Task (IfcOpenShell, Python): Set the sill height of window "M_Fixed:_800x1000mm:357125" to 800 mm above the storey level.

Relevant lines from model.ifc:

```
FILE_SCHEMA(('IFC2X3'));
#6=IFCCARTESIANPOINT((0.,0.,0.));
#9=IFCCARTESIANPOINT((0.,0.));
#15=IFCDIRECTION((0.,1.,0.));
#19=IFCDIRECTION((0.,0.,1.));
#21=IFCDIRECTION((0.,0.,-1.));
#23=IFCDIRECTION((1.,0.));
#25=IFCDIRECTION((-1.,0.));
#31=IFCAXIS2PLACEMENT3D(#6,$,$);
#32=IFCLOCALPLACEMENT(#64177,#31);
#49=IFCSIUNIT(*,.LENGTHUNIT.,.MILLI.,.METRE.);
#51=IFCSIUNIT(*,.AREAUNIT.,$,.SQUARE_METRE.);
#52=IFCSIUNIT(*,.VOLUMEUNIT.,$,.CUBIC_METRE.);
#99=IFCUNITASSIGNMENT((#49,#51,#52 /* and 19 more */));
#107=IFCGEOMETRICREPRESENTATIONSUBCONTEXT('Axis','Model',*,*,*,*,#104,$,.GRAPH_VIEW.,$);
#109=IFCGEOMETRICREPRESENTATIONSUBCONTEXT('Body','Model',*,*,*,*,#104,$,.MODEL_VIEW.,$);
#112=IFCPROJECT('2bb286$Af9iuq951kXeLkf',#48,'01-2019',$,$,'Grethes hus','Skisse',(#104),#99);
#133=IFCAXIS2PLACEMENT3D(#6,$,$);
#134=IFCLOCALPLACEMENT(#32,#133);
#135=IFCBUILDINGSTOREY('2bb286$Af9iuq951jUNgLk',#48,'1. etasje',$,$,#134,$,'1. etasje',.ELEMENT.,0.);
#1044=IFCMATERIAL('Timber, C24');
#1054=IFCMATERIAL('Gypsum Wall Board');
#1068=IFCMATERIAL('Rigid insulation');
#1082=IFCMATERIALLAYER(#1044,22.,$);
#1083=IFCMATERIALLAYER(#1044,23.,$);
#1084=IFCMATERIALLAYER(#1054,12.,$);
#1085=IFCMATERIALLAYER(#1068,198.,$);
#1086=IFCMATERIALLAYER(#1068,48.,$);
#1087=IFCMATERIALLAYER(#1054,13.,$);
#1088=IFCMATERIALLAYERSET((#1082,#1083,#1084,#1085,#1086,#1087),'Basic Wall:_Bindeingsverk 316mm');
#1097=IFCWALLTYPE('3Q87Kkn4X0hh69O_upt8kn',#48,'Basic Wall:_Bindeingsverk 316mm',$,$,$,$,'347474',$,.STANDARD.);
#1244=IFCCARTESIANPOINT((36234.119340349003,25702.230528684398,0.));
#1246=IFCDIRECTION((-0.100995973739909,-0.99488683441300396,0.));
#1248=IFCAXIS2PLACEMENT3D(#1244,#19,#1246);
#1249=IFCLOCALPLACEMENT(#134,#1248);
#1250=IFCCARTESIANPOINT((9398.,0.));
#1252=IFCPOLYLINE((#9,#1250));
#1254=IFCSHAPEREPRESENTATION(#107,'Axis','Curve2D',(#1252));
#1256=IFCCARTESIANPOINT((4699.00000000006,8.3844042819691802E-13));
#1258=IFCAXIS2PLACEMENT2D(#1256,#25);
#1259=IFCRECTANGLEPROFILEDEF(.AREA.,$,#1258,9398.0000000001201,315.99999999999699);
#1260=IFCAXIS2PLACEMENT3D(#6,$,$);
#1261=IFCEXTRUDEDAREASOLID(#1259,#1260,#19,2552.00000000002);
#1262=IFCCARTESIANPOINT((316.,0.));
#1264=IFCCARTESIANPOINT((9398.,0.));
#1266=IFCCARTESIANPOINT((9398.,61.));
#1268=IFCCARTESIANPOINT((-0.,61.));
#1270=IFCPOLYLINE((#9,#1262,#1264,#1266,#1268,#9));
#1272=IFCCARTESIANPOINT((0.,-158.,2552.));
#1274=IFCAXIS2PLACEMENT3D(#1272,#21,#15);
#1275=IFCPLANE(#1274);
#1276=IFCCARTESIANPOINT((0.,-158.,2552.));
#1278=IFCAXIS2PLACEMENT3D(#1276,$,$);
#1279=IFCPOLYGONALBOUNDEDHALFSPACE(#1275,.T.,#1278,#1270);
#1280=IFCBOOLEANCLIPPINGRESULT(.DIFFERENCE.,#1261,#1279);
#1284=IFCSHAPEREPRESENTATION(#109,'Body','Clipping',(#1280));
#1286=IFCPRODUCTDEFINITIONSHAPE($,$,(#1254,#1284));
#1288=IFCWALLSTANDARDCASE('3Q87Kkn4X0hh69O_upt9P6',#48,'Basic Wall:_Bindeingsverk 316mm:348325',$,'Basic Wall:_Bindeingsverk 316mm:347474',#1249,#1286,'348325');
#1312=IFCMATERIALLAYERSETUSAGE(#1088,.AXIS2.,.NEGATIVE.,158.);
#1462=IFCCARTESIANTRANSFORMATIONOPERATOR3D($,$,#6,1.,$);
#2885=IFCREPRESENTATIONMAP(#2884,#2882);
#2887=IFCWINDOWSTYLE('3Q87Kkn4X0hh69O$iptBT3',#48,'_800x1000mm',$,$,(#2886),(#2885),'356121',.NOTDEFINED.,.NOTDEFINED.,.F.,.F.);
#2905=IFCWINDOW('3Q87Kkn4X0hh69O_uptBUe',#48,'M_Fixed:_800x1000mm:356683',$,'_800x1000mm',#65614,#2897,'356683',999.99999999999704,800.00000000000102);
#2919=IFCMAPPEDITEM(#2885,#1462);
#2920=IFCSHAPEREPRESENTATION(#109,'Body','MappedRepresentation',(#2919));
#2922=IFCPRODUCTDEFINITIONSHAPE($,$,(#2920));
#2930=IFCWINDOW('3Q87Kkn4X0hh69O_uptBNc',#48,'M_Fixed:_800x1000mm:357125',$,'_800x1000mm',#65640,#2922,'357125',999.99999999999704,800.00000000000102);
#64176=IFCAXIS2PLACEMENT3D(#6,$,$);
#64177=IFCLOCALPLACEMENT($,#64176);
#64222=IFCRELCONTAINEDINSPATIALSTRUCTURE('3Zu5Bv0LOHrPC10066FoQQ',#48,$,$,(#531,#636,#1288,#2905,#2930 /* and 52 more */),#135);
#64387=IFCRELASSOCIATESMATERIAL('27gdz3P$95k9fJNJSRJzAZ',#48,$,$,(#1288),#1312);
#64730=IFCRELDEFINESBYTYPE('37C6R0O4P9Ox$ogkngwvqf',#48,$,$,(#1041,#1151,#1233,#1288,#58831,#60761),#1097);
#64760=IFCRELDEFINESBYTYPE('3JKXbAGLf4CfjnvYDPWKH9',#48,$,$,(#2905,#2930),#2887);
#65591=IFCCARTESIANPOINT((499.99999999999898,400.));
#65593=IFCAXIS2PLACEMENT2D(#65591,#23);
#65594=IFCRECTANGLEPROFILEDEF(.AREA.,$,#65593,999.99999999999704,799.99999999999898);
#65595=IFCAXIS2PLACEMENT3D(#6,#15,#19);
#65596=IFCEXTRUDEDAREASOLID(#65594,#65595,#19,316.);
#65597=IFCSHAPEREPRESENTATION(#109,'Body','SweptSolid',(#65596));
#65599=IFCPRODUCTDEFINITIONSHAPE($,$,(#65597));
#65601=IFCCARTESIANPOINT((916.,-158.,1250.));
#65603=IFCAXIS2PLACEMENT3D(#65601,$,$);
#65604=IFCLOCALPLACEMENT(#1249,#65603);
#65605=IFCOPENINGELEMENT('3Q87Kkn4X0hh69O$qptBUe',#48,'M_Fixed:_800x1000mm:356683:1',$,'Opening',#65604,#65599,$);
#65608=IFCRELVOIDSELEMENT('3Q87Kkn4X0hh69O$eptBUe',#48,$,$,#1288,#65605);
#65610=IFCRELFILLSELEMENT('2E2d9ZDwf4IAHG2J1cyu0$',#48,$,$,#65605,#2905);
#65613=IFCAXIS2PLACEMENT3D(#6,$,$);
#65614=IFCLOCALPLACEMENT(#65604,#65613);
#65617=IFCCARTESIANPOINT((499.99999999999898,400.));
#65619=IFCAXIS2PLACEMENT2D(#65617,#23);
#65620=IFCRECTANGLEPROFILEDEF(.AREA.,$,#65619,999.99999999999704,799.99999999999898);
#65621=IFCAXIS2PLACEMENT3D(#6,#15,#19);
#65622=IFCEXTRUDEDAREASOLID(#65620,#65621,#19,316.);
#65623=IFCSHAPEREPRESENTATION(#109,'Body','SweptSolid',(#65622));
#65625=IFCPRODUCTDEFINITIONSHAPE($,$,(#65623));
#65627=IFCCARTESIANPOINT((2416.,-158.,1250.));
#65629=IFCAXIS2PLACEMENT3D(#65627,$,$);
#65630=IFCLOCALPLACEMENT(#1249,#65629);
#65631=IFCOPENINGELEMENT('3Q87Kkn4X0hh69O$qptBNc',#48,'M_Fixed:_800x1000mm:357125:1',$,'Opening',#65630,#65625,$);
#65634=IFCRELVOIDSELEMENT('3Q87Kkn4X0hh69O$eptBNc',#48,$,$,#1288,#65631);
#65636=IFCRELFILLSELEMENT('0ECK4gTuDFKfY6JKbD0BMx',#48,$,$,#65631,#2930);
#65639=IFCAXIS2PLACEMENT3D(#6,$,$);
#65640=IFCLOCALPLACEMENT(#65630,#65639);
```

```python
import numpy as np
import ifcopenshell
import ifcopenshell.api.geometry
import ifcopenshell.geom
import ifcopenshell.util.element
import ifcopenshell.util.placement
import ifcopenshell.util.shape
import ifcopenshell.util.unit

model = ifcopenshell.open("model.ifc")
unit_scale = ifcopenshell.util.unit.calculate_unit_scale(model)

window = model.by_guid("3Q87Kkn4X0hh69O_uptBNc")
opening = window.FillsVoids[0].RelatingOpeningElement
storey = ifcopenshell.util.element.get_container(window, ifc_class="IfcBuildingStorey")
level = ifcopenshell.util.placement.get_local_placement(storey.ObjectPlacement)[2, 3]

# The opening's origin need not be at the sill, so measure its lowest point.
shape = ifcopenshell.geom.create_shape(ifcopenshell.geom.settings(), opening)
bottom = ifcopenshell.util.shape.get_shape_bottom_elevation(shape, shape.geometry) / unit_scale
dz = level + 800.0 - bottom

shift = np.array([0.0, 0.0, dz])
# The window is placed relative to its opening, so it follows when the opening moves.
matrix = ifcopenshell.util.placement.get_local_placement(opening.ObjectPlacement)
matrix[:3, 3] += shift
ifcopenshell.api.geometry.edit_object_placement(
    model, product=opening, matrix=matrix, is_si=False, should_transform_children=True
)

print(f"moved by {dz * unit_scale:+.3f} m")

model.write("model_rev.ifc")
```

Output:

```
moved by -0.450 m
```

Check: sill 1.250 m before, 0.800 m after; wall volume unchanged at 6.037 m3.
